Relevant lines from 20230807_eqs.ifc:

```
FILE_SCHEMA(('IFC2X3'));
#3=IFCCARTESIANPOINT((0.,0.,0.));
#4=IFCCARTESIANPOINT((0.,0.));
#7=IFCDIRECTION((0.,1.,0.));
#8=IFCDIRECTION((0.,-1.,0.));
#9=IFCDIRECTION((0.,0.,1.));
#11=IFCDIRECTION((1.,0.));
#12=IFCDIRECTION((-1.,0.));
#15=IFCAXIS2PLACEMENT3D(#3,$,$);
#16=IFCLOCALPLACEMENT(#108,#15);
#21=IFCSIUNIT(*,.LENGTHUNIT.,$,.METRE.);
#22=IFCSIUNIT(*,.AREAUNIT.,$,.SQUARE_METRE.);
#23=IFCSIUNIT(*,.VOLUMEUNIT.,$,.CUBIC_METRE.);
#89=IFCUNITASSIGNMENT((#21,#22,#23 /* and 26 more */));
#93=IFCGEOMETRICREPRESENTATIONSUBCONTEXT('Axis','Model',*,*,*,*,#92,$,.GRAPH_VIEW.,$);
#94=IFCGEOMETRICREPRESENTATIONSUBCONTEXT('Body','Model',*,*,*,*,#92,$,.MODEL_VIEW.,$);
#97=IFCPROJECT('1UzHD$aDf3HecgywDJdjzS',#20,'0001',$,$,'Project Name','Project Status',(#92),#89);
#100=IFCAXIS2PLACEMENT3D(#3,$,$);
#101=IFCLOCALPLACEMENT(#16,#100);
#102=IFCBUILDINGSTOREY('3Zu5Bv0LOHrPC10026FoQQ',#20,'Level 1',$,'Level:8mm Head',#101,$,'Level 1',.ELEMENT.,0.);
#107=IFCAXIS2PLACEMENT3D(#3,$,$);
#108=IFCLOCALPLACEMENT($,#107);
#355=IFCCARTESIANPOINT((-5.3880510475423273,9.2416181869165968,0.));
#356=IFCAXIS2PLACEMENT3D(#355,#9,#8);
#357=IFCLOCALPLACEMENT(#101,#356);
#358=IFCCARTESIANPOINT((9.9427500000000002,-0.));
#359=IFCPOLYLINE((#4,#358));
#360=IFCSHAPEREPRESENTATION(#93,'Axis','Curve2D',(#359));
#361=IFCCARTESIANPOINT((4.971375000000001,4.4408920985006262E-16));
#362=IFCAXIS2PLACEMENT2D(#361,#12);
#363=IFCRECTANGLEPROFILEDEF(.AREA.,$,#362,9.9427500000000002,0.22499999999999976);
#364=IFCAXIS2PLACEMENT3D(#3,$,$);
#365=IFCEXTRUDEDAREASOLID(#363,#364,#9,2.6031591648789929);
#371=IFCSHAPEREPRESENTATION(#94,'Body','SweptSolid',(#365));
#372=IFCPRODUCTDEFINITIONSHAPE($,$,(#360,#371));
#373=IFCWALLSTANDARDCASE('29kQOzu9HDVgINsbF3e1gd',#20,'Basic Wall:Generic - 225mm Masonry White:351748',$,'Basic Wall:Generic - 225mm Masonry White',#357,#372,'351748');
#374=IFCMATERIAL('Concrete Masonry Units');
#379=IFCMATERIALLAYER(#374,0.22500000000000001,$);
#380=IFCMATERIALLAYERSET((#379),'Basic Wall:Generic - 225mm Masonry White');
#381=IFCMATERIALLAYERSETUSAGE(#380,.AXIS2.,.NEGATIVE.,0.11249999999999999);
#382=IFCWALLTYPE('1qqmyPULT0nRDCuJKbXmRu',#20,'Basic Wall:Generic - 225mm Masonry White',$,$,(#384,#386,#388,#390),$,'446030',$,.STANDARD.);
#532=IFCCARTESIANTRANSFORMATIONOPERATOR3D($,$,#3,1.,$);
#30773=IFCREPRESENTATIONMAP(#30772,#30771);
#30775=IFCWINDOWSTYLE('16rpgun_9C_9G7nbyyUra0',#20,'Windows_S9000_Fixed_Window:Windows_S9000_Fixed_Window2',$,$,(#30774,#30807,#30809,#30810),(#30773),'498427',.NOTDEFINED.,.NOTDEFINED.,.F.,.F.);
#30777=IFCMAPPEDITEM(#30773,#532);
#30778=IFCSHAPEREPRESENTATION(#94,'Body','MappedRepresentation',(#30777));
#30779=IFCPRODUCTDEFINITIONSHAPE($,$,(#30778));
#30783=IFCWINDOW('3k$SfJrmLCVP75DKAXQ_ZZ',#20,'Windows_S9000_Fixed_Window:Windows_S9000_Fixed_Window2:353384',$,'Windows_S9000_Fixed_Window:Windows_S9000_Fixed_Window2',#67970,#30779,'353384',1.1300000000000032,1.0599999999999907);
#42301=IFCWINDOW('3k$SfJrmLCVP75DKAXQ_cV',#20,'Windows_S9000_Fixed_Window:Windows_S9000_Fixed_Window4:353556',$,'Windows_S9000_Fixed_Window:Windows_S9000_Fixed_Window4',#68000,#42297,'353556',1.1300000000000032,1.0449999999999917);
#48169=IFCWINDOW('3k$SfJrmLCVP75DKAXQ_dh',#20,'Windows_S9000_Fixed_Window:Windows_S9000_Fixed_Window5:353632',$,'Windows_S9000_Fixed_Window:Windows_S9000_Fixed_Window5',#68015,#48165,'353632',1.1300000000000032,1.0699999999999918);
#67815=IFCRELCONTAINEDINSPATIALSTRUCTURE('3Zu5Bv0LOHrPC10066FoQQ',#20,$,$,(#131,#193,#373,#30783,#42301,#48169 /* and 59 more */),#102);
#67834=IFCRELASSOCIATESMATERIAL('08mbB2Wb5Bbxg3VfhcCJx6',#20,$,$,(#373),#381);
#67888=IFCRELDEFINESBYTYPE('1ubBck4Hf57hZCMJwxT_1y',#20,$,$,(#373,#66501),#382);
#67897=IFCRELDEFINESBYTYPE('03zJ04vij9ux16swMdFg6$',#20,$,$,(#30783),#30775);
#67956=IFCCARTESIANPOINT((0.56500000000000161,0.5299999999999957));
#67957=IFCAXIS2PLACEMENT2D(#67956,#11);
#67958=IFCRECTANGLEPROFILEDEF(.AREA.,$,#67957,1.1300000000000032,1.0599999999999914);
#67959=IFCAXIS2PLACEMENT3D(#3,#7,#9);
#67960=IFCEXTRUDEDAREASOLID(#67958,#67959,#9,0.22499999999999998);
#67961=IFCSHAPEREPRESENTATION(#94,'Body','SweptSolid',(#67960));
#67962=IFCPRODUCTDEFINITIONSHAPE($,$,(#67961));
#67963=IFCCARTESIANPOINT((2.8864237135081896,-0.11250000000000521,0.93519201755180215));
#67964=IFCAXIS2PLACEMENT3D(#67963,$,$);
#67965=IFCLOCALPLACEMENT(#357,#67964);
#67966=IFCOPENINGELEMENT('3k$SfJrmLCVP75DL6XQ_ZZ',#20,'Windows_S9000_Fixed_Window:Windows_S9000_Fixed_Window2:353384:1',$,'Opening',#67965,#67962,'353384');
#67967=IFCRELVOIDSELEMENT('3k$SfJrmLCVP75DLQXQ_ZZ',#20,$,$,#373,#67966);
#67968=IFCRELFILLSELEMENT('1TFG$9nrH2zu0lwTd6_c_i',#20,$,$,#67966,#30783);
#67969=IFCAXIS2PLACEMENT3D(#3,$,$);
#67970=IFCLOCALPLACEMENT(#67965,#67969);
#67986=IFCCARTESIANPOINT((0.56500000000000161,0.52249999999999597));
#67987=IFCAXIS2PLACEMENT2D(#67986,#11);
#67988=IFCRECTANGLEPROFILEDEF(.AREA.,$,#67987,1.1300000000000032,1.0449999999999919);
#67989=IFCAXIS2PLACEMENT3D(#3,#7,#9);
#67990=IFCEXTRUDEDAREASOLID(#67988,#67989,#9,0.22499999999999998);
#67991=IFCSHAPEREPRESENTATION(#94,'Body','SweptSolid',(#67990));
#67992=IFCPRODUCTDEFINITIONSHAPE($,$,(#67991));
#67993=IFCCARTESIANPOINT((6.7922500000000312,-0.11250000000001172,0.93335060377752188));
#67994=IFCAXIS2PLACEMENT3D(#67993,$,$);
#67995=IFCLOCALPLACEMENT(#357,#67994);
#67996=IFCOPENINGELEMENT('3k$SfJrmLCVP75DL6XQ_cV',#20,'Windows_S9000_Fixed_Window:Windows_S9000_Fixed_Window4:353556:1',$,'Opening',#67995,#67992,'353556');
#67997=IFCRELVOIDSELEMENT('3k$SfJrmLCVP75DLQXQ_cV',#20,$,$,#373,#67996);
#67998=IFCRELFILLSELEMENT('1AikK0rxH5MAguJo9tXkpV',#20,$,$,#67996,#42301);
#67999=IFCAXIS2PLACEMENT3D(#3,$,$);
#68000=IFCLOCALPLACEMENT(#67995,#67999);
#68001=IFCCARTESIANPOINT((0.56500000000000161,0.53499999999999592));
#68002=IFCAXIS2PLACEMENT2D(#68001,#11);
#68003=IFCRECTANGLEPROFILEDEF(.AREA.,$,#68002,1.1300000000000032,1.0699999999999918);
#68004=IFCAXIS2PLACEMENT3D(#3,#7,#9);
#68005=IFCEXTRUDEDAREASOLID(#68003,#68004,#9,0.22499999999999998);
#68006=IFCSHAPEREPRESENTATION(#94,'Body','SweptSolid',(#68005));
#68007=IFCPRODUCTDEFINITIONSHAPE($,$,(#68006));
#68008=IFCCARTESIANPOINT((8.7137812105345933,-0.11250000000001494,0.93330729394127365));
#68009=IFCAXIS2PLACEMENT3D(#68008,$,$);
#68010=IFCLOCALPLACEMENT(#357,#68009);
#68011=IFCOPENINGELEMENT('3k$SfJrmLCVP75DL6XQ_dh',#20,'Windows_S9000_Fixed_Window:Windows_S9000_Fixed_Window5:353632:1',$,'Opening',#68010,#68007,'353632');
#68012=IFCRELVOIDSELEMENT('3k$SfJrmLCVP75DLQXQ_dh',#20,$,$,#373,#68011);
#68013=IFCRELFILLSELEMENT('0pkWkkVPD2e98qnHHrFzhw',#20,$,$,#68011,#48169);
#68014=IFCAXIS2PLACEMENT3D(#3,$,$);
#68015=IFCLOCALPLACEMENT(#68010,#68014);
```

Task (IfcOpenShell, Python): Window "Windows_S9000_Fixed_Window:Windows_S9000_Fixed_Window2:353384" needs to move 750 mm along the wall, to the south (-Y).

```python
import ifcopenshell
import ifcopenshell.api.geometry
import ifcopenshell.util.placement
import ifcopenshell.util.unit

model = ifcopenshell.open("20230807_eqs.ifc")
unit_scale = ifcopenshell.util.unit.calculate_unit_scale(model)

window = model.by_id(30783)
opening = window.FillsVoids[0].RelatingOpeningElement
wall = opening.VoidsElements[0].RelatingBuildingElement

wall_matrix = ifcopenshell.util.placement.get_local_placement(wall.ObjectPlacement)
shift = wall_matrix[:3, 0] * 0.75 / unit_scale
before = ifcopenshell.util.placement.get_local_placement(window.ObjectPlacement)[:3, 3].copy()

# The window is placed relative to its opening, so it follows when the opening moves.
matrix = ifcopenshell.util.placement.get_local_placement(opening.ObjectPlacement)
matrix[:3, 3] += shift
ifcopenshell.api.geometry.edit_object_placement(
    model, product=opening, matrix=matrix, is_si=False, should_transform_children=True
)

after = ifcopenshell.util.placement.get_local_placement(window.ObjectPlacement)[:3, 3]
print("window moved by", (after - before).round(3) + 0.0)

model.write("20230807_eqs-out.ifc")
```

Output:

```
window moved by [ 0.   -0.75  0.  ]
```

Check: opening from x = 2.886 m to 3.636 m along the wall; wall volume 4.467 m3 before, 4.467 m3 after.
